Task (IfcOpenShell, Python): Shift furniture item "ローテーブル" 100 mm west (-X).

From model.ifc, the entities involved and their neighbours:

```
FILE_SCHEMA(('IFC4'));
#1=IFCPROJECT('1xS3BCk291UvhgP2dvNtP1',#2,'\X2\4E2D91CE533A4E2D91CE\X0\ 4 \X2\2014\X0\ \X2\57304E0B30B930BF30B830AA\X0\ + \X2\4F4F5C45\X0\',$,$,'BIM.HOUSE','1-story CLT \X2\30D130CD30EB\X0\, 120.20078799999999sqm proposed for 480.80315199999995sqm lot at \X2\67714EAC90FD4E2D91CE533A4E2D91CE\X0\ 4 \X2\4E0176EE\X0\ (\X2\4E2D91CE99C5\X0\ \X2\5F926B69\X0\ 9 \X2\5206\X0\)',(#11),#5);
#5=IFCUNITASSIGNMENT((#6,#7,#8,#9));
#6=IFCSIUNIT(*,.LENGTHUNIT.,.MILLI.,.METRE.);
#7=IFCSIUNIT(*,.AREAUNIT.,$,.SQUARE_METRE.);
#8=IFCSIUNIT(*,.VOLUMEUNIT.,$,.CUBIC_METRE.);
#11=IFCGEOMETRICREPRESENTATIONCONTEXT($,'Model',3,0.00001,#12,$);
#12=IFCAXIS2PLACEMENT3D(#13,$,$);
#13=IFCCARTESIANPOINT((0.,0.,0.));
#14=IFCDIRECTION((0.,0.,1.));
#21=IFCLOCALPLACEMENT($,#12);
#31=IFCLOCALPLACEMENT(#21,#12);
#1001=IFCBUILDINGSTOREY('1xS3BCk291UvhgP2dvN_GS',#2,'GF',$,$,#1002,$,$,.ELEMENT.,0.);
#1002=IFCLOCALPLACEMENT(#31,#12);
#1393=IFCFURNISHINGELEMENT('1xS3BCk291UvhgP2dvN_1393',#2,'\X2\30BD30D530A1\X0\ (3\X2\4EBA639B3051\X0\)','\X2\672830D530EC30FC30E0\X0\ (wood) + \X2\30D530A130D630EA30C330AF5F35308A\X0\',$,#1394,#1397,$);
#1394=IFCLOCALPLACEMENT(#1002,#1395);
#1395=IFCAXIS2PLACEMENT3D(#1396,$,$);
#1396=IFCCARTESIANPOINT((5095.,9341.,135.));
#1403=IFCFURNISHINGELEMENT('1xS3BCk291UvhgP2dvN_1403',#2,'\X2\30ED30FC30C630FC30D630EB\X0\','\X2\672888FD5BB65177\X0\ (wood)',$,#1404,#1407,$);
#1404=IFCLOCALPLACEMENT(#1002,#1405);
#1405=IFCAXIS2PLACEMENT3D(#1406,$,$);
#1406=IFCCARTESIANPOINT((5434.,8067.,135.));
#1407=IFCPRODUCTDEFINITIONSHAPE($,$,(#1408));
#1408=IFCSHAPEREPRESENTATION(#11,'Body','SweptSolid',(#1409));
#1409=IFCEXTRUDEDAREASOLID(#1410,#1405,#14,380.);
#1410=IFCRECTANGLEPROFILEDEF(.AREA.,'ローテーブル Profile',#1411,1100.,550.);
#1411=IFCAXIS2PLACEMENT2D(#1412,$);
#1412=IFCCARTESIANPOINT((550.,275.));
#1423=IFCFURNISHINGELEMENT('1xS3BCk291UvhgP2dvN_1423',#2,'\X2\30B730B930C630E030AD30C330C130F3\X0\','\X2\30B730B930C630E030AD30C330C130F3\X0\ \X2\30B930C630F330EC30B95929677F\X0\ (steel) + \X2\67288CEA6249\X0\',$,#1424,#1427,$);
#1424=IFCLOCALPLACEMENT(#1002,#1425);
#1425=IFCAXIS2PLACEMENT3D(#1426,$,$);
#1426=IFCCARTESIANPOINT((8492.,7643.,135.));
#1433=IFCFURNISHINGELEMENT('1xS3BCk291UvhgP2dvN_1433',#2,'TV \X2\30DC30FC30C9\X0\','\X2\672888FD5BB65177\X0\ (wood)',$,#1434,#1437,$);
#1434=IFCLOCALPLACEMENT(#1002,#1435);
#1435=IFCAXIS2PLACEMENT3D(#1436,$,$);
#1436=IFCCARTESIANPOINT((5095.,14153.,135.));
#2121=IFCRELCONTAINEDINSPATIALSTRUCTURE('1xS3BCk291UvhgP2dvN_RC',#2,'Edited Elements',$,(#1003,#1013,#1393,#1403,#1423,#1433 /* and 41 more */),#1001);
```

```python
import ifcopenshell
import ifcopenshell.api.geometry
import ifcopenshell.util.placement
import ifcopenshell.util.unit

model = ifcopenshell.open("model.ifc")
unit_scale = ifcopenshell.util.unit.calculate_unit_scale(model)

item = model.by_guid("1xS3BCk291UvhgP2dvN_1403")
matrix = ifcopenshell.util.placement.get_local_placement(item.ObjectPlacement)
matrix[0, 3] -= 0.1 / unit_scale
ifcopenshell.api.geometry.edit_object_placement(model, product=item, matrix=matrix, is_si=False)

print(ifcopenshell.util.placement.get_local_placement(item.ObjectPlacement).round(3) + 0.0)

model.write("model_edited.ifc")
```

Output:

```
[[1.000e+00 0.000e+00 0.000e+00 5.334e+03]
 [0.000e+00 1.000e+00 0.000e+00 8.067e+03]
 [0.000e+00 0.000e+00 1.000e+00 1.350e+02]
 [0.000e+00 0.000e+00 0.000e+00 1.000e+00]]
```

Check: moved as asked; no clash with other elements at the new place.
